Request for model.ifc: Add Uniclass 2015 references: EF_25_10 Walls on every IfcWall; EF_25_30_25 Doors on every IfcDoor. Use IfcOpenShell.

First a look at what the model holds.

```python
import ifcopenshell

model = ifcopenshell.open("model.ifc")
print(model.schema)
print("classifications:", [c.Name for c in model.by_type("IfcClassification")])
for ifc_class in ("IfcDoor", "IfcRoof", "IfcStair", "IfcWall", "IfcWindow"):
    print(ifc_class, len(model.by_type(ifc_class)))
```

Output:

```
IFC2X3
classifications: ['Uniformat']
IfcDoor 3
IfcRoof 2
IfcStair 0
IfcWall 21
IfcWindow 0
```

```python
import ifcopenshell
import ifcopenshell.api.classification

model = ifcopenshell.open("model.ifc")

# IFC2X3 requires Source and Edition and has no link from the project to the system.
system = model.create_entity("IfcClassification", Source="NBS", Edition="2015", Name="Uniclass 2015")

codes = {
    "IfcWall": ("EF_25_10", "Walls"),
    "IfcDoor": ("EF_25_30_25", "Doors"),
}
for ifc_class, (code, name) in codes.items():
    products = model.by_type(ifc_class)
    ifcopenshell.api.classification.add_reference(
        model, products=products, classification=system, identification=code, name=name
    )
    print(code, len(products))

model.write("model-out.ifc")
```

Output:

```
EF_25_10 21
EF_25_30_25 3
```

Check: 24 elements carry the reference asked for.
